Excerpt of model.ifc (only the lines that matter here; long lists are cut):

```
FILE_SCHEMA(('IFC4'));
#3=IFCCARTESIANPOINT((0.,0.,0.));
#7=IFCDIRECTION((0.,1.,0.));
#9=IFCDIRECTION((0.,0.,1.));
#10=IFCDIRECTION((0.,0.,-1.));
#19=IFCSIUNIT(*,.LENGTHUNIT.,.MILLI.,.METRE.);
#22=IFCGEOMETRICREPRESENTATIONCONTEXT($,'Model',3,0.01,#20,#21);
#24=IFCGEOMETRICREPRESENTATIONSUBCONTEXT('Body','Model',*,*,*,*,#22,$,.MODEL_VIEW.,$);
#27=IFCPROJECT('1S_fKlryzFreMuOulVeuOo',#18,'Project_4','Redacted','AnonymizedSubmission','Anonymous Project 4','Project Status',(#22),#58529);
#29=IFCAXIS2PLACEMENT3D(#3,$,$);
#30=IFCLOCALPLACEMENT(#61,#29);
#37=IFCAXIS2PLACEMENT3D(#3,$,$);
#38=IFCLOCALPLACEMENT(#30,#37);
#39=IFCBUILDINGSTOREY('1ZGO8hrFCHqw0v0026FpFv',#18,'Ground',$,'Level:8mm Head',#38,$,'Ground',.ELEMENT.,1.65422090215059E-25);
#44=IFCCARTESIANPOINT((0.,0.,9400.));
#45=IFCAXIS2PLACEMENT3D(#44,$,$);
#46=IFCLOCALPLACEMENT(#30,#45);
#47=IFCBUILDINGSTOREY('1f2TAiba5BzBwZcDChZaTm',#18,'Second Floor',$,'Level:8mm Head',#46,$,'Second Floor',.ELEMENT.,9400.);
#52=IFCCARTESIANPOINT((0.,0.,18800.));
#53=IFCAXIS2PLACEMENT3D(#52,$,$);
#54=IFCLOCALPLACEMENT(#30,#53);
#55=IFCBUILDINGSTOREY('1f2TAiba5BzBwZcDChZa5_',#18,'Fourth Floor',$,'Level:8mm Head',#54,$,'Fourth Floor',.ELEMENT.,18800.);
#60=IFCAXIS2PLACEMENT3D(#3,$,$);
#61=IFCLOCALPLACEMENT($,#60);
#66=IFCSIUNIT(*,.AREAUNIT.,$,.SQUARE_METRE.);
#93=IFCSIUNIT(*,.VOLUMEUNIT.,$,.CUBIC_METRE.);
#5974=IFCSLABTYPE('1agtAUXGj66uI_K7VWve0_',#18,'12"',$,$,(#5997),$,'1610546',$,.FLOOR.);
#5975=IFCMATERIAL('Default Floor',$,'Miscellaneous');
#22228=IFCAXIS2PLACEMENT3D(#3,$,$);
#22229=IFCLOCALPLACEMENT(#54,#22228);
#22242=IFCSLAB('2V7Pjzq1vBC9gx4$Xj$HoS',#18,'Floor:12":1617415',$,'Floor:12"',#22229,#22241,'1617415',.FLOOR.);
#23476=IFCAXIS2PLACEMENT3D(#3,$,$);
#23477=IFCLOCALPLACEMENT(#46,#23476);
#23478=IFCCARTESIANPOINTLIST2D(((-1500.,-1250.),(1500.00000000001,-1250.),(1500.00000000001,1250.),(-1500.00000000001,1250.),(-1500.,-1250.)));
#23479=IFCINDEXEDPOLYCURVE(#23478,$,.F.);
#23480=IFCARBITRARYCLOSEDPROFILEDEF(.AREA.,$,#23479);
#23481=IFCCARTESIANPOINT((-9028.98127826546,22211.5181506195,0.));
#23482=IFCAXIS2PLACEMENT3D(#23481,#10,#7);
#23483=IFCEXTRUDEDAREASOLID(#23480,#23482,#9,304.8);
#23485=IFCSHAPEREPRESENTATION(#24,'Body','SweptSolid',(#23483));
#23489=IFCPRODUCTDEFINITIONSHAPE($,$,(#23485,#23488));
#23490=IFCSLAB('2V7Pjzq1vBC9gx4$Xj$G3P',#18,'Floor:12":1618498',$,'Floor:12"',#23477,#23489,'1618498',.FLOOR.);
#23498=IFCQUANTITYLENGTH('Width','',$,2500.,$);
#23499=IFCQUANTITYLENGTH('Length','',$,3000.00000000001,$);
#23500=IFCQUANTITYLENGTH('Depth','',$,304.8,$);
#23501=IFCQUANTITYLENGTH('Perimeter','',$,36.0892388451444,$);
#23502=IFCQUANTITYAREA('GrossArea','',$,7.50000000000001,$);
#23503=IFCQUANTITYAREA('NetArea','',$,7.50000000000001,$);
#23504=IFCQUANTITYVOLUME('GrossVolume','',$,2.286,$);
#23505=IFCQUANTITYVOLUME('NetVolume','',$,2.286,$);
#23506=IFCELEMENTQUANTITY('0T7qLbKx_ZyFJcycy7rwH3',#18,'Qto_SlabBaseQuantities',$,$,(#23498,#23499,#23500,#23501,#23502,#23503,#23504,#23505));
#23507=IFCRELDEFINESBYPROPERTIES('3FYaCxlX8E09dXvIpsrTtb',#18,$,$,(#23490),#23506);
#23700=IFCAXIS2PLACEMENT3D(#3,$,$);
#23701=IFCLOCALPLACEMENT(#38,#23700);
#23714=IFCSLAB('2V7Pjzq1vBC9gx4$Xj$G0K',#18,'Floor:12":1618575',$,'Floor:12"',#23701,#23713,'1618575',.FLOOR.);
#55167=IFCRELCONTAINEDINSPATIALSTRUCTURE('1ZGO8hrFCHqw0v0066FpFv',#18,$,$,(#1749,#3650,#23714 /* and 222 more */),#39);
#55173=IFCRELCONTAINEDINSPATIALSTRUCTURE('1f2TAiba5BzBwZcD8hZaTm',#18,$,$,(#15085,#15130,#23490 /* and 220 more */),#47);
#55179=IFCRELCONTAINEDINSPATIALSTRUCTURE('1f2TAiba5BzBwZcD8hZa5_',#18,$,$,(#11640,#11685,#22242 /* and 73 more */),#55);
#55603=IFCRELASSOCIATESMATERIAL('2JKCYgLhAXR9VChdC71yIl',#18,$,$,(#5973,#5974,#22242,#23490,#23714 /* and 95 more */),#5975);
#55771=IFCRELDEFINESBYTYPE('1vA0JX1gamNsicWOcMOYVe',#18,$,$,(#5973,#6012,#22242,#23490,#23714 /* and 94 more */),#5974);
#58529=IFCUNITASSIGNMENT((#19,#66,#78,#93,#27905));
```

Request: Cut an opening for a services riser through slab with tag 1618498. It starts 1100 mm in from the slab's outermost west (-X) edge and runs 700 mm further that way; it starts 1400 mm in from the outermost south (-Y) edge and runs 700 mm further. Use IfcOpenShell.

```python
import numpy as np
import ifcopenshell
import ifcopenshell.api.feature
import ifcopenshell.api.geometry
import ifcopenshell.api.pset
import ifcopenshell.api.root
import ifcopenshell.geom
import ifcopenshell.util.element
import ifcopenshell.util.placement
import ifcopenshell.util.representation
import ifcopenshell.util.shape
import ifcopenshell.util.unit

model = ifcopenshell.open("model.ifc")
unit_scale = ifcopenshell.util.unit.calculate_unit_scale(model)
area_scale = ifcopenshell.util.unit.calculate_unit_scale(model, "AREAUNIT")
volume_scale = ifcopenshell.util.unit.calculate_unit_scale(model, "VOLUMEUNIT")
settings = ifcopenshell.geom.settings()


def volume(element):
    """Net volume in cubic metres, openings subtracted."""
    shape = ifcopenshell.geom.create_shape(settings, element)
    return ifcopenshell.util.shape.get_volume(shape.geometry)


slab = model.by_guid("2V7Pjzq1vBC9gx4$Xj$G3P")
before = volume(slab)

# Extent in the slab's own axes, in metres. The edges named are its -X and -Y sides.
slab_shape = ifcopenshell.geom.create_shape(settings, slab)
vertices = ifcopenshell.util.shape.get_vertices(slab_shape.geometry)
x_min, y_min, bottom = vertices.min(axis=0)
top = vertices[:, 2].max()

opening = ifcopenshell.api.root.create_entity(model, ifc_class="IfcOpeningElement", name="Services riser opening", predefined_type="OPENING")
context = ifcopenshell.util.representation.get_context(model, "Model", "Body", "MODEL_VIEW")
width, depth = 0.7, 0.7
outline = [(0.0, 0.0), (width, 0.0), (width, depth), (0.0, depth), (0.0, 0.0)]
# Overshoot both faces by 50 mm so the cut is clean.
shape = ifcopenshell.api.geometry.add_slab_representation(
    model, context=context, depth=top - bottom + 0.1, polyline=outline
)
ifcopenshell.api.geometry.assign_representation(model, product=opening, representation=shape)

matrix = ifcopenshell.util.placement.get_local_placement(slab.ObjectPlacement)
matrix[:, 3] = matrix @ np.append(np.array([x_min + 1.1, y_min + 1.4, bottom - 0.05]) / unit_scale, 1.0)
ifcopenshell.api.geometry.edit_object_placement(model, product=opening, matrix=matrix, is_si=False)
ifcopenshell.api.feature.add_feature(model, feature=opening, element=slab)

after = volume(slab)

# Update the slab's stored quantities.
qto = model.by_id(ifcopenshell.util.element.get_pset(slab, "Qto_SlabBaseQuantities", should_inherit=False)["id"])
ifcopenshell.api.pset.edit_qto(model, qto=qto, properties={
    "NetArea": after / (top - bottom) / area_scale,
    "NetVolume": after / volume_scale,
})

print(f"slab volume {before:.3f} -> {after:.3f} m3")

model.write("model_updated.ifc")
```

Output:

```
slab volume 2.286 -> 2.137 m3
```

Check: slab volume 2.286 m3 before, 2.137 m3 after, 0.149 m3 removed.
